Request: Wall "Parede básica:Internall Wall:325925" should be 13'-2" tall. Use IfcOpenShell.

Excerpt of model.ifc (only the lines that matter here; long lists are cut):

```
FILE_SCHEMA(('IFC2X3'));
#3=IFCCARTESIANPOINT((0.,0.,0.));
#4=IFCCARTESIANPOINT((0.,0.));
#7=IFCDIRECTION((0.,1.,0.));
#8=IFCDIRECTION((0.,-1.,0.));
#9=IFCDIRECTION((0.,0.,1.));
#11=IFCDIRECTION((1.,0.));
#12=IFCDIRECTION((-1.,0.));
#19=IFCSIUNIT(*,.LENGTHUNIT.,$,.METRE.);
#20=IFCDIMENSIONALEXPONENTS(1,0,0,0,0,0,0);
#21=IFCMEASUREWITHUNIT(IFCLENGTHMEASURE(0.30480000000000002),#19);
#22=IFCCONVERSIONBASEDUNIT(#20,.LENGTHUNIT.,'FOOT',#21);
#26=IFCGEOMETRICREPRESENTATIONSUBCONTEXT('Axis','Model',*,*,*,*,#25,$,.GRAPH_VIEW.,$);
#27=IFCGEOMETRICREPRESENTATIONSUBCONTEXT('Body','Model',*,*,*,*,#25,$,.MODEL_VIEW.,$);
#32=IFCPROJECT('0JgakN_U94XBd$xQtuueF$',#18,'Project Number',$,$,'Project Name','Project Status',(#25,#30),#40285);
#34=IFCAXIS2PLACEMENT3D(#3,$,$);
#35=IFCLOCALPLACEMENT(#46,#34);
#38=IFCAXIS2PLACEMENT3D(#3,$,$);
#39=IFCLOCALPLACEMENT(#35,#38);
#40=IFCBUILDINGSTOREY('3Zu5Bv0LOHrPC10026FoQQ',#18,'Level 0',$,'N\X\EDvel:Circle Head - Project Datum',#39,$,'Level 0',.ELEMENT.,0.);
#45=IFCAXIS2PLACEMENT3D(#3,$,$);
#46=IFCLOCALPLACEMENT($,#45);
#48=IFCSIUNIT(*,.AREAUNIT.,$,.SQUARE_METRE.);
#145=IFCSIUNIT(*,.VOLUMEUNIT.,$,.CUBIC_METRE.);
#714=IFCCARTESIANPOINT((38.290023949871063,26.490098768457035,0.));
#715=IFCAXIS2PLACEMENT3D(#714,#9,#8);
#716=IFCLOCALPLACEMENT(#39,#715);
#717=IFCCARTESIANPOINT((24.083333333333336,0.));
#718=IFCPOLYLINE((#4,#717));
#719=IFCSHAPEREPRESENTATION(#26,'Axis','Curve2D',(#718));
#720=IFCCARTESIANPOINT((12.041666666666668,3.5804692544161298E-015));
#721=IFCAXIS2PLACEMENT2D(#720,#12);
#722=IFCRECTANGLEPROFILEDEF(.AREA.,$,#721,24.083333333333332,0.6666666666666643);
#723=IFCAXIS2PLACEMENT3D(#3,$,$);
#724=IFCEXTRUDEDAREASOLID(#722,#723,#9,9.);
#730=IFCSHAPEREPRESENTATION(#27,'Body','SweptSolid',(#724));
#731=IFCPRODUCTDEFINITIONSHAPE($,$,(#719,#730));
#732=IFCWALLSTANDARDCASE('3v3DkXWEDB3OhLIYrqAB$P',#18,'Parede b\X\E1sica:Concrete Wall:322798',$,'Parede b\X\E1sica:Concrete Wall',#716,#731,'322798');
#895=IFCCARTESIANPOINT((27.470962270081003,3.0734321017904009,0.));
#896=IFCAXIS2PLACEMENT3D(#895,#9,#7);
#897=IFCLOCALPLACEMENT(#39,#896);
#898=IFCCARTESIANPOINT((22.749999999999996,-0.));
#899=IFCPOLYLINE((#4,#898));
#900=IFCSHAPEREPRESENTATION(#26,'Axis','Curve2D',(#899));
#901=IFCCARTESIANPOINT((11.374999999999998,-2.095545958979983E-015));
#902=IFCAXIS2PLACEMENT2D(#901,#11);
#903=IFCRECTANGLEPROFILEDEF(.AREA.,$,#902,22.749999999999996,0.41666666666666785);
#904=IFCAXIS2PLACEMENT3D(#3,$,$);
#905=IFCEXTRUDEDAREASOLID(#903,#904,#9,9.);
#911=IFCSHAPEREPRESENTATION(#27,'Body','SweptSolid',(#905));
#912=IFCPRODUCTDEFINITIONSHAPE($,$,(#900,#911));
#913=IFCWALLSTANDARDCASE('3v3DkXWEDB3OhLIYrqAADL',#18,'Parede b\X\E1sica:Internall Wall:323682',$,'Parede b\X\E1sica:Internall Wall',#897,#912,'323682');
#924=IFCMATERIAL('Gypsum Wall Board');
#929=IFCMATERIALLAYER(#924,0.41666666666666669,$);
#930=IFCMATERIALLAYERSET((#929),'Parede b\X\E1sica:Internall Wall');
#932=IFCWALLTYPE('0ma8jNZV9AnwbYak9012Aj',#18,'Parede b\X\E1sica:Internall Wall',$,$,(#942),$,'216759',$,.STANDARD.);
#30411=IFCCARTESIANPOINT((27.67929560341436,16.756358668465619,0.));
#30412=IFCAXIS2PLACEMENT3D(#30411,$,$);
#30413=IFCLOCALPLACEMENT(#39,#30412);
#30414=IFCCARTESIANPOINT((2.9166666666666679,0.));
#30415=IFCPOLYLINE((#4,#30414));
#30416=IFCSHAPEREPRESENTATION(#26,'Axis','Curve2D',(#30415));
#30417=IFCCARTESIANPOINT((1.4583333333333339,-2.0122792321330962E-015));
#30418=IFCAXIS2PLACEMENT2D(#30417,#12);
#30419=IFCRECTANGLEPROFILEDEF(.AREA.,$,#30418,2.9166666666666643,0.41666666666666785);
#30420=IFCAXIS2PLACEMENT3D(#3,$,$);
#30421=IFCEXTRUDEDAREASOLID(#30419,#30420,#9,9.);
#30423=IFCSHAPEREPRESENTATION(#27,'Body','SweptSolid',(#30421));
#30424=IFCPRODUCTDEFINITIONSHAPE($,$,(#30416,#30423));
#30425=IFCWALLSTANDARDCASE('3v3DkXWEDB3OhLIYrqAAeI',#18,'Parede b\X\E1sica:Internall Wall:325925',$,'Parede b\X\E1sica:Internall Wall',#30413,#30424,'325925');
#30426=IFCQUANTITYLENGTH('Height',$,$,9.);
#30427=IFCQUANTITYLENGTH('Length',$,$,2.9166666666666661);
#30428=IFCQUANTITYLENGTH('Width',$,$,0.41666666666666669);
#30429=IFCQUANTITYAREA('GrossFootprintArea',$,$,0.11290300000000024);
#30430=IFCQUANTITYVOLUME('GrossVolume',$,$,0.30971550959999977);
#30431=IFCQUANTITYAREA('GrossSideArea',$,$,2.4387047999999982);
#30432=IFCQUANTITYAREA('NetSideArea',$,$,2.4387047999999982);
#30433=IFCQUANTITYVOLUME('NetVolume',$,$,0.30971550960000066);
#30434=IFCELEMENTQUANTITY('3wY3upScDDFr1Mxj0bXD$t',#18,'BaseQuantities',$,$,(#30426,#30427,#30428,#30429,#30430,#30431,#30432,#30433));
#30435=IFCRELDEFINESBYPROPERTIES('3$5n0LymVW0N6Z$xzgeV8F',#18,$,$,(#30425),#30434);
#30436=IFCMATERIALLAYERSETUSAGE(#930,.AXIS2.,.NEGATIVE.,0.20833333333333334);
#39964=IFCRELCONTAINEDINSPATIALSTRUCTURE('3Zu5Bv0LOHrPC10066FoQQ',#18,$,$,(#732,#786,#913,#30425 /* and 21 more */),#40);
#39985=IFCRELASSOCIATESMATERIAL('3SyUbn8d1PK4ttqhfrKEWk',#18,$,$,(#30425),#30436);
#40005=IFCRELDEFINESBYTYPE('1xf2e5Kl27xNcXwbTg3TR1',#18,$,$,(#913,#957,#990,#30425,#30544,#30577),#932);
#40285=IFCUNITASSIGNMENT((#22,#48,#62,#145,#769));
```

```python
import ifcopenshell
import ifcopenshell.api.pset
import ifcopenshell.geom
import ifcopenshell.util.element
import ifcopenshell.util.representation
import ifcopenshell.util.shape
import ifcopenshell.util.unit

model = ifcopenshell.open("model.ifc")
unit_scale = ifcopenshell.util.unit.calculate_unit_scale(model)
area_scale = ifcopenshell.util.unit.calculate_unit_scale(model, "AREAUNIT")
volume_scale = ifcopenshell.util.unit.calculate_unit_scale(model, "VOLUMEUNIT")
settings = ifcopenshell.geom.settings()


def volume(element):
    """Net volume in cubic metres, openings subtracted."""
    shape = ifcopenshell.geom.create_shape(settings, element)
    return ifcopenshell.util.shape.get_volume(shape.geometry)


wall = model.by_guid("3v3DkXWEDB3OhLIYrqAAeI")
before = volume(wall)

body = ifcopenshell.util.representation.get_representation(wall, "Model", "Body")
solid = body.Items[0]
old_height = solid.Depth
solid.Depth = 158 * 0.0254 / unit_scale
after = volume(wall)
thickness = 0.127  # wall thickness in metres

# Update the stored height, areas and volumes.
qto = model.by_id(ifcopenshell.util.element.get_pset(wall, "BaseQuantities", should_inherit=False)["id"])
ifcopenshell.api.pset.edit_qto(model, qto=qto, properties={
    "Height": solid.Depth,
    "GrossVolume": ifcopenshell.util.element.get_pset(wall, "BaseQuantities", "GrossVolume") * solid.Depth / old_height,
    "GrossSideArea": ifcopenshell.util.element.get_pset(wall, "BaseQuantities", "GrossSideArea") * solid.Depth / old_height,
    "NetSideArea": after / thickness / area_scale,
    "NetVolume": after / volume_scale,
})

print(f"height {old_height:g} -> {solid.Depth:g}, volume {before:.3f} -> {after:.3f} m3")

model.write("model_rev.ifc")
```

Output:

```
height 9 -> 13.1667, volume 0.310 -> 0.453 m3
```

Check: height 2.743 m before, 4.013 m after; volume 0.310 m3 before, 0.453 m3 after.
